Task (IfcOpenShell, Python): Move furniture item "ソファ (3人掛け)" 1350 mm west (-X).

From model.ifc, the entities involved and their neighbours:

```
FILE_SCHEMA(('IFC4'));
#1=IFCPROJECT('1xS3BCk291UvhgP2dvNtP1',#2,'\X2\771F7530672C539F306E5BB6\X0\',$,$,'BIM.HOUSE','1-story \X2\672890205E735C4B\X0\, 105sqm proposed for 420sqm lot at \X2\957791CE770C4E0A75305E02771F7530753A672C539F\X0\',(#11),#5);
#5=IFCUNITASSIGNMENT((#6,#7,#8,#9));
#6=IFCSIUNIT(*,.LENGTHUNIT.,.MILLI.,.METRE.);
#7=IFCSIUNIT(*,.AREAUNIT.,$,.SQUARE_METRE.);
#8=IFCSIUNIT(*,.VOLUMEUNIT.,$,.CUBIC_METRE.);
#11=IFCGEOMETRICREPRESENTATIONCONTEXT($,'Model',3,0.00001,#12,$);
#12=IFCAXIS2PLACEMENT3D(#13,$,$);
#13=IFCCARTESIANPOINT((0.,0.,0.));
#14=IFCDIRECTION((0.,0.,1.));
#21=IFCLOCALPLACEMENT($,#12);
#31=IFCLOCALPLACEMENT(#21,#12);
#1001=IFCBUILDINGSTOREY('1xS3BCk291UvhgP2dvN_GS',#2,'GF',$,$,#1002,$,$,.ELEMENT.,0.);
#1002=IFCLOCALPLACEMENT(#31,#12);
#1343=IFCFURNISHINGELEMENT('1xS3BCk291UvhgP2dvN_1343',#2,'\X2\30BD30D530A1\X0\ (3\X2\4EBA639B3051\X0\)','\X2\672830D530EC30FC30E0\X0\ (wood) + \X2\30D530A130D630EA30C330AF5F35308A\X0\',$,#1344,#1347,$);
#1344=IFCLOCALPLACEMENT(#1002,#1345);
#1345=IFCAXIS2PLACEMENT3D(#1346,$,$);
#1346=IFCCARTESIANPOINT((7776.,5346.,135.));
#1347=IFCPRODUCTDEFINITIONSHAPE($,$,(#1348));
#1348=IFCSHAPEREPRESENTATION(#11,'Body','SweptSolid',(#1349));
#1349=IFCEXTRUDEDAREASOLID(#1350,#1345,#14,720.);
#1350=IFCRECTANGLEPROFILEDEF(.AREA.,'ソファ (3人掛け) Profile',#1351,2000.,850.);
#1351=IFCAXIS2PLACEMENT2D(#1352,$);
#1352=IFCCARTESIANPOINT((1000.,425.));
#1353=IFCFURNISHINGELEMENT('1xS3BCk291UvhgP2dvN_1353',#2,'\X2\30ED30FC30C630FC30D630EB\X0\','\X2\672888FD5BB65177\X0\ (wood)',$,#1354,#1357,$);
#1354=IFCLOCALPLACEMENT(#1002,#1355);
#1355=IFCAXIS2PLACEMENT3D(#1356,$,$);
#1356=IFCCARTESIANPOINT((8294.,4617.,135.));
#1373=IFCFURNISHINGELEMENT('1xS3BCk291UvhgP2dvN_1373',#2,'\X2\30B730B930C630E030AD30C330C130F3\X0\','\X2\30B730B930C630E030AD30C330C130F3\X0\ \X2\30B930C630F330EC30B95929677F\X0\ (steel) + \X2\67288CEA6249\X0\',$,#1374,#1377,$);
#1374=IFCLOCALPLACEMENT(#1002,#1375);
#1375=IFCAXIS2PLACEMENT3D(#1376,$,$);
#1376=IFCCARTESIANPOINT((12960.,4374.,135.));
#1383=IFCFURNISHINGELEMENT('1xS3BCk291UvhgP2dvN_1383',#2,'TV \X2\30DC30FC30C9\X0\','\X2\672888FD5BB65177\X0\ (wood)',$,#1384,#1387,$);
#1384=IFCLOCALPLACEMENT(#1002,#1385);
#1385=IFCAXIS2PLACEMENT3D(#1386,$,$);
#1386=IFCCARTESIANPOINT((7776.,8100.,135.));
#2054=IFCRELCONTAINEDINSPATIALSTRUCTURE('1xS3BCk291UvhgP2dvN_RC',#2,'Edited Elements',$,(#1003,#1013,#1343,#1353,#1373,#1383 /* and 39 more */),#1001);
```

```python
import ifcopenshell
import ifcopenshell.api.geometry
import ifcopenshell.util.placement

model = ifcopenshell.open("model.ifc")

item = model.by_guid("1xS3BCk291UvhgP2dvN_1343")
matrix = ifcopenshell.util.placement.get_local_placement(item.ObjectPlacement)
matrix[0, 3] -= 1350.0
ifcopenshell.api.geometry.edit_object_placement(model, product=item, matrix=matrix, is_si=False)

print(ifcopenshell.util.placement.get_local_placement(item.ObjectPlacement).round(3) + 0.0)

model.write("model_edited.ifc")
```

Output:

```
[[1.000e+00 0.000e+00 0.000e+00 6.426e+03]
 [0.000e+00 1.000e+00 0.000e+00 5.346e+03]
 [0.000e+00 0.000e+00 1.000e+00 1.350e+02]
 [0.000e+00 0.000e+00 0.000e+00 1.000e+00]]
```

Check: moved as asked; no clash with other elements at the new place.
